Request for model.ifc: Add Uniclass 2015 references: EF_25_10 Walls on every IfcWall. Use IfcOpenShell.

First a look at what the model holds.

```python
import ifcopenshell

model = ifcopenshell.open("model.ifc")
print(model.schema)
print("classifications:", [c.Name for c in model.by_type("IfcClassification")])
for ifc_class in ("IfcDoor", "IfcRoof", "IfcStair", "IfcWall", "IfcWindow"):
    print(ifc_class, len(model.by_type(ifc_class)))
```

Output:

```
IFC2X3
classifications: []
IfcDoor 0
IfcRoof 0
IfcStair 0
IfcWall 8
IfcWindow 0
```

```python
import ifcopenshell
import ifcopenshell.api.classification

model = ifcopenshell.open("model.ifc")

# IFC2X3 requires Source and Edition and has no link from the project to the system.
system = model.create_entity("IfcClassification", Source="NBS", Edition="2015", Name="Uniclass 2015")

codes = {
    "IfcWall": ("EF_25_10", "Walls"),
}
for ifc_class, (code, name) in codes.items():
    products = model.by_type(ifc_class)
    ifcopenshell.api.classification.add_reference(
        model, products=products, classification=system, identification=code, name=name
    )
    print(code, len(products))

model.write("model_v2.ifc")
```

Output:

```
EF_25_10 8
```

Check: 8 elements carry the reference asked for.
